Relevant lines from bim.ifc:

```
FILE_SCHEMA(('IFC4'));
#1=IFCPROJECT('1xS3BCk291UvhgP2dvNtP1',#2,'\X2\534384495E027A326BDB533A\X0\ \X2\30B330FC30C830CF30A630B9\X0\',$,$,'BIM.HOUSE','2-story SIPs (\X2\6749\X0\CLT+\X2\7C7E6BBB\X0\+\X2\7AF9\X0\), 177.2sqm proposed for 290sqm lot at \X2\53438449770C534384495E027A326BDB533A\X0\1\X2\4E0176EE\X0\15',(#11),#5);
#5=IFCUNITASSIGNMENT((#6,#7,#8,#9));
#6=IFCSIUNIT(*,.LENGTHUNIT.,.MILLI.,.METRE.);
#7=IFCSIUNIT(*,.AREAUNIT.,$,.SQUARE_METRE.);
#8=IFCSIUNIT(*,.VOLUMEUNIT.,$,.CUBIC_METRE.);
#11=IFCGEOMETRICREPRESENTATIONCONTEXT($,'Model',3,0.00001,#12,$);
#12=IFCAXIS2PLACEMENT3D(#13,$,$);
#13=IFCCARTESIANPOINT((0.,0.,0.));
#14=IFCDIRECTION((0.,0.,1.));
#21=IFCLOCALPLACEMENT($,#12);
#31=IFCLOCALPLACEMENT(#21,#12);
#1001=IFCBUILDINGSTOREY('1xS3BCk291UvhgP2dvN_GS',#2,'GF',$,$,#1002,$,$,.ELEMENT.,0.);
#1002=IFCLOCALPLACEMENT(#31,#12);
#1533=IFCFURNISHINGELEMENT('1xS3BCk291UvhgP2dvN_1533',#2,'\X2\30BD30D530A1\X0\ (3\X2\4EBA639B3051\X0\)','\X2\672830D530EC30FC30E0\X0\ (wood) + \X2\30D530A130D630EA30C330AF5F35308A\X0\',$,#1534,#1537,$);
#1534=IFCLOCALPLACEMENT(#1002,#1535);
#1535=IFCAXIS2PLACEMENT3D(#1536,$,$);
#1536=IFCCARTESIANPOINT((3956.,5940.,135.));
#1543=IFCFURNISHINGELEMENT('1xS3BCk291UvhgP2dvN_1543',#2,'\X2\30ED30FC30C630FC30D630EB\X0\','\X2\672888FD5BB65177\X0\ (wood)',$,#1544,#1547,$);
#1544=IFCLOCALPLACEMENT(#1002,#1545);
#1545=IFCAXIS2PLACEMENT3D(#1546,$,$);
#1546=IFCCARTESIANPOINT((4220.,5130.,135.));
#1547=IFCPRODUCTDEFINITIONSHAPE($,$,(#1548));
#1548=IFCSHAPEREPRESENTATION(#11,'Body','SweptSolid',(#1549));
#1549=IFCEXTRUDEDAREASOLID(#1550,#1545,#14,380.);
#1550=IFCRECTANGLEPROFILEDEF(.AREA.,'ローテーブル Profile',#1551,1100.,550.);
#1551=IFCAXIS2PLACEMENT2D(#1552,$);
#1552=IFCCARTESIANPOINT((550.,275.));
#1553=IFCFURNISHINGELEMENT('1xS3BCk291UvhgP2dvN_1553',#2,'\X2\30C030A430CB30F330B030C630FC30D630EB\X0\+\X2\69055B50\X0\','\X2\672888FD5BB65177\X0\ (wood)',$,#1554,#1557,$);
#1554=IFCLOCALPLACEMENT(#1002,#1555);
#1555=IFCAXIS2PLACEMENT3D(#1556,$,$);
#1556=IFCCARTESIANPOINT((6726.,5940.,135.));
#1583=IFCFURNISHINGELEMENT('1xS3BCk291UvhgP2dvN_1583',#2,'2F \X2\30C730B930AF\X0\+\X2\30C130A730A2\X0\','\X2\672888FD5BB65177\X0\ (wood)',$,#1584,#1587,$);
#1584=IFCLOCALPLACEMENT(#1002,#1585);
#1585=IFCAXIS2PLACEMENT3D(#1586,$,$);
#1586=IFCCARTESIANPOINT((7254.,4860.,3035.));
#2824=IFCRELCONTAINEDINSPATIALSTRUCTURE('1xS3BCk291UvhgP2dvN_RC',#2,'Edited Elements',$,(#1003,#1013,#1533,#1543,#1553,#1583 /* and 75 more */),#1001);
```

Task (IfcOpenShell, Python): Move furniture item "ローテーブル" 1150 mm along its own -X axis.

```python
import ifcopenshell
import ifcopenshell.api.geometry
import ifcopenshell.util.placement

model = ifcopenshell.open("bim.ifc")

item = model.by_guid("1xS3BCk291UvhgP2dvN_1543")
matrix = ifcopenshell.util.placement.get_local_placement(item.ObjectPlacement)
matrix[:3, 3] -= matrix[:3, 0] * 1150.0
ifcopenshell.api.geometry.edit_object_placement(model, product=item, matrix=matrix, is_si=False)

print(ifcopenshell.util.placement.get_local_placement(item.ObjectPlacement).round(3) + 0.0)

model.write("bim_v2.ifc")
```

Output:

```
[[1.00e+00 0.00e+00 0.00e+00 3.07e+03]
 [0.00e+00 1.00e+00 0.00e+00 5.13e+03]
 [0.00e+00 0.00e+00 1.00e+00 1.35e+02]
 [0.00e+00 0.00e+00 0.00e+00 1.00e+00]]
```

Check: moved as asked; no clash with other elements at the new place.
